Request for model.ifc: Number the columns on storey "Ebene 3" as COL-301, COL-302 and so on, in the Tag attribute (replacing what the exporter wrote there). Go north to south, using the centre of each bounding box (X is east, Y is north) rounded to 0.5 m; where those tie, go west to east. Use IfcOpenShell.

First a look at what the model holds.

```python
import ifcopenshell
import ifcopenshell.util.element
import ifcopenshell.util.placement

model = ifcopenshell.open("model.ifc")
print(model.schema)
storey = next(s for s in model.by_type("IfcBuildingStorey") if s.Name == "Ebene 3")
columns = [e for e in ifcopenshell.util.element.get_decomposition(storey) if e.is_a("IfcColumn")]
for e in sorted(columns, key=lambda e: e.id()):
    origin = ifcopenshell.util.placement.get_local_placement(e.ObjectPlacement)[:3, 3]
    print(e.id(), e.Tag, e.Name, origin.round(2) + 0.0, sep=" | ")
```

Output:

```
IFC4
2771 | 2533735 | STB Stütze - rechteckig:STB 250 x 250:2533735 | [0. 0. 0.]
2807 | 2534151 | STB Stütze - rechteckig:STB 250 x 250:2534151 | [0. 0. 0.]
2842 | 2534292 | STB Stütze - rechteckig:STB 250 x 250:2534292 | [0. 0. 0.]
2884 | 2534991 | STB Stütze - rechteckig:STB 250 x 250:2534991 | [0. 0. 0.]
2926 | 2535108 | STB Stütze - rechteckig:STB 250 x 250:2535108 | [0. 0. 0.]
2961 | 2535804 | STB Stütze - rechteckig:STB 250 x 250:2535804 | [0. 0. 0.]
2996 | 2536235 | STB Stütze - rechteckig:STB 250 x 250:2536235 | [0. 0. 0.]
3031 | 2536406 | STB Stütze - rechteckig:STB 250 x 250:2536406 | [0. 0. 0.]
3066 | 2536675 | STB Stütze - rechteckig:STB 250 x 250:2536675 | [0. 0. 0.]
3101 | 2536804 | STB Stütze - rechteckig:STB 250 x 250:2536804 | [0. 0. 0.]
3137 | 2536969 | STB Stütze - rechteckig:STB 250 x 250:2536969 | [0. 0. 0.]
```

```python
import ifcopenshell
import ifcopenshell.geom
import ifcopenshell.util.element
import ifcopenshell.util.shape

model = ifcopenshell.open("model.ifc")
settings = ifcopenshell.geom.settings()
settings.set("use-world-coords", True)


def centre(element):
    shape = ifcopenshell.geom.create_shape(settings, element)
    return ifcopenshell.util.shape.get_bbox_centroid(shape.geometry)


storey = next(s for s in model.by_type("IfcBuildingStorey") if s.Name == "Ebene 3")
columns = [e for e in ifcopenshell.util.element.get_decomposition(storey) if e.is_a("IfcColumn")]

# Insertion points can sit at a corner or the storey origin, so sort by the geometry (in metres).
centres = {e: centre(e) for e in columns}
columns.sort(key=lambda e: (-round(centres[e][1] / 0.5), centres[e][0]))

for i, e in enumerate(columns, start=1):
    number = f"COL-3{i:02d}"
    e.Tag = number
    print(e.id(), number)

model.write("model_v2.ifc")
```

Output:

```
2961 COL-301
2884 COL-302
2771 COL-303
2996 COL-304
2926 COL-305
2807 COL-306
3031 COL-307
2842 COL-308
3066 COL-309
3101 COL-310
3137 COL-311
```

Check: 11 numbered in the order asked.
